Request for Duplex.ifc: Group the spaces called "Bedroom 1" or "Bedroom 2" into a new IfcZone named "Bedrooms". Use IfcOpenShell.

First a look at what the model holds.

```python
import ifcopenshell

model = ifcopenshell.open("Duplex.ifc")
print(model.schema)
seen = {}
for space in model.by_type("IfcSpace"):
    seen[space.LongName] = seen.get(space.LongName, 0) + 1
for name, count in sorted(seen.items(), key=str):
    print(count, "x", name)
print("zones:", [z.Name for z in model.by_type("IfcZone")][:20])
```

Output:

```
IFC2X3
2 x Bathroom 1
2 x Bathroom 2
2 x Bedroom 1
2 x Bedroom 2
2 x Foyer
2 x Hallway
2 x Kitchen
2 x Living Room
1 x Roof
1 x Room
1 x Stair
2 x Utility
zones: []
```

```python
import ifcopenshell
import ifcopenshell.api.group
import ifcopenshell.api.root

model = ifcopenshell.open("Duplex.ifc")

names = {"Bedroom 1", "Bedroom 2"}
spaces = [s for s in model.by_type("IfcSpace") if s.LongName in names]

zone = ifcopenshell.api.root.create_entity(model, ifc_class="IfcZone", name="Bedrooms")
ifcopenshell.api.group.assign_group(model, products=spaces, group=zone)
print(len(spaces), "spaces in", zone.Name)

model.write("Duplex_rev.ifc")
```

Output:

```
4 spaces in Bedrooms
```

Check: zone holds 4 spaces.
